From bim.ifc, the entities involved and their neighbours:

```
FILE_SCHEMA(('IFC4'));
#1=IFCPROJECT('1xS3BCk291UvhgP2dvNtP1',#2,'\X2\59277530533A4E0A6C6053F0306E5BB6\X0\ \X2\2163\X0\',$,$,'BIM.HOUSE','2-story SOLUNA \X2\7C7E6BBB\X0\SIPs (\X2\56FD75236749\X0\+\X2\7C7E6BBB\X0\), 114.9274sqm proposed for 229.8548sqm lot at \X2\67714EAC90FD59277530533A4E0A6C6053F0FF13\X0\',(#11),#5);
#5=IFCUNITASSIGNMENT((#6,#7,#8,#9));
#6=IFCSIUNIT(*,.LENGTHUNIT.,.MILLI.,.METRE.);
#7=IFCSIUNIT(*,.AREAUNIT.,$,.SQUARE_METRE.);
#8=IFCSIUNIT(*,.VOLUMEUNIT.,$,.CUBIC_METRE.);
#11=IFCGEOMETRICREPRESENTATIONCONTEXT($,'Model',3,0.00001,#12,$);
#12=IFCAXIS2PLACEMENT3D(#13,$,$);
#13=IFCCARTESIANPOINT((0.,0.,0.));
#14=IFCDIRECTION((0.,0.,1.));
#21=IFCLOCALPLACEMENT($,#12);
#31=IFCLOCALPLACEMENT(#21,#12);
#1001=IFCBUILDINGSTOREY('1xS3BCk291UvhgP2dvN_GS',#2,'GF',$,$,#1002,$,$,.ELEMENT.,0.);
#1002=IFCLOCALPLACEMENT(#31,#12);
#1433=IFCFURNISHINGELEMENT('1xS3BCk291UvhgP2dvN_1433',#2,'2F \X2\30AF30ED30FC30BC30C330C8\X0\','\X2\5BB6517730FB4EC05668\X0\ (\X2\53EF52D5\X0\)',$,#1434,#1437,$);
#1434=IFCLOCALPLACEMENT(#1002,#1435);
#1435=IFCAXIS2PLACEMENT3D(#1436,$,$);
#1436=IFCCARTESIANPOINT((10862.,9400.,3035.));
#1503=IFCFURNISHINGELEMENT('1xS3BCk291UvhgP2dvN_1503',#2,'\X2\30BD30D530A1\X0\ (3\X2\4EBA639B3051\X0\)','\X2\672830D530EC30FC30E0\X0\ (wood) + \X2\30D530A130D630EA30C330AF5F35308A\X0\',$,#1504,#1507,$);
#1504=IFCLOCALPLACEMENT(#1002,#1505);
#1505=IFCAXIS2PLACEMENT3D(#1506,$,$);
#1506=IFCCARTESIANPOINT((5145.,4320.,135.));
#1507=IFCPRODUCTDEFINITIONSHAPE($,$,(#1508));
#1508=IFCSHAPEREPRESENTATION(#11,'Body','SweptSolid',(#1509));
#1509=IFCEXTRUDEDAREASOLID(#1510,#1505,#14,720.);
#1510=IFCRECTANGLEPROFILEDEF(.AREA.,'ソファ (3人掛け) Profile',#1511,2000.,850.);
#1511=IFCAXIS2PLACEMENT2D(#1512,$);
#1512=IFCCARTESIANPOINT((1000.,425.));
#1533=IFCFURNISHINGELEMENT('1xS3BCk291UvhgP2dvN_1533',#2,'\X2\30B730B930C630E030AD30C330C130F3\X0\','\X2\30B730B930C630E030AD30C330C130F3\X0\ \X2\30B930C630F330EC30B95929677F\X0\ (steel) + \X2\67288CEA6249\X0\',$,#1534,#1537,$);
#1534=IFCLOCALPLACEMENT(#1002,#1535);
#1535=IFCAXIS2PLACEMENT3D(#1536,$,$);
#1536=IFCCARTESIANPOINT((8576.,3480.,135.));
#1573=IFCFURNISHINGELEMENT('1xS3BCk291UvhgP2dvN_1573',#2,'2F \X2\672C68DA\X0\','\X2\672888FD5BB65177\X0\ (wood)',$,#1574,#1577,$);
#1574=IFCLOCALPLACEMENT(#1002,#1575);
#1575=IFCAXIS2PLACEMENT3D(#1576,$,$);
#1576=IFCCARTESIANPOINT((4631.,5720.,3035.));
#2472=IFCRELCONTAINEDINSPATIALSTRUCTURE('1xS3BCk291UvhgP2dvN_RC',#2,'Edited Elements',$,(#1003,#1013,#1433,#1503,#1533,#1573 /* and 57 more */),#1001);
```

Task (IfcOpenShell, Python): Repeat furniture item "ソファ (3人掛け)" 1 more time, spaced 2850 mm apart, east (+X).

```python
import numpy as np
import ifcopenshell
import ifcopenshell.api.geometry
import ifcopenshell.api.root
import ifcopenshell.util.element
import ifcopenshell.util.placement

model = ifcopenshell.open("bim.ifc")


def reuse_history(source, copy):
    """copy_class also copies each property set's owner history, people and application; keep the originals."""
    for rel in copy.IsDefinedBy:
        if rel.is_a("IfcRelDefinesByProperties") and (history := rel.RelatingPropertyDefinition.OwnerHistory):
            rel.RelatingPropertyDefinition.OwnerHistory = source.OwnerHistory
            ifcopenshell.util.element.remove_deep2(model, history)


source = model.by_id(1503)
base = ifcopenshell.util.placement.get_local_placement(source.ObjectPlacement)
step = np.array([1.0, 0.0, 0.0]) * 2850.0

for i in range(1, 2):
    copy = ifcopenshell.api.root.copy_class(model, product=source)
    copy.Representation = ifcopenshell.util.element.copy_deep(
        model, source.Representation, exclude=["IfcGeometricRepresentationContext", "IfcRepresentationMap"]
    )
    reuse_history(source, copy)
    matrix = base.copy()
    matrix[:3, 3] += i * step
    print("added at", matrix[:3, 3].round(3) + 0.0)
    ifcopenshell.api.geometry.edit_object_placement(model, product=copy, matrix=matrix, is_si=False)

model.write("bim-out.ifc")
```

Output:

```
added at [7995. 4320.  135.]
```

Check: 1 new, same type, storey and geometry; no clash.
